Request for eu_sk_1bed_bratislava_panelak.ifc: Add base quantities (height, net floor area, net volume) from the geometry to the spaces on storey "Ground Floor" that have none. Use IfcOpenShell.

First a look at what the model holds.

```python
import ifcopenshell
import ifcopenshell.util.element
import ifcopenshell.util.unit

model = ifcopenshell.open("eu_sk_1bed_bratislava_panelak.ifc")
print(model.schema)
for unit_type in ("LENGTHUNIT", "AREAUNIT", "VOLUMEUNIT"):
    print(unit_type, ifcopenshell.util.unit.calculate_unit_scale(model, unit_type))
storey = next(s for s in model.by_type("IfcBuildingStorey") if s.Name == "Ground Floor")
spaces = [e for e in ifcopenshell.util.element.get_decomposition(storey) if e.is_a("IfcSpace")]
for e in sorted(spaces, key=lambda e: e.id()):
    print(e.id(), e.is_a(), e.Name, list(ifcopenshell.util.element.get_psets(e, qtos_only=True)), sep=" | ")
```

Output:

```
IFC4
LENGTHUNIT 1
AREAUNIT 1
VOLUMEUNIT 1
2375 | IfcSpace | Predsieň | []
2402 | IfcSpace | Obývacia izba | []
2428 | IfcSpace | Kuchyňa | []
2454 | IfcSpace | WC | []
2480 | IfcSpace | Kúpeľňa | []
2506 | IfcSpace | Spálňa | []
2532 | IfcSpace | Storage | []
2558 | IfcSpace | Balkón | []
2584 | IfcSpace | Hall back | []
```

```python
import ifcopenshell
import ifcopenshell.api.pset
import ifcopenshell.geom
import ifcopenshell.util.element
import ifcopenshell.util.shape
import ifcopenshell.util.unit

model = ifcopenshell.open("eu_sk_1bed_bratislava_panelak.ifc")
unit_scale = ifcopenshell.util.unit.calculate_unit_scale(model)
area_scale = ifcopenshell.util.unit.calculate_unit_scale(model, "AREAUNIT")
volume_scale = ifcopenshell.util.unit.calculate_unit_scale(model, "VOLUMEUNIT")
settings = ifcopenshell.geom.settings()

storey = next(s for s in model.by_type("IfcBuildingStorey") if s.Name == "Ground Floor")
spaces = [e for e in ifcopenshell.util.element.get_decomposition(storey) if e.is_a("IfcSpace")]

for e in sorted(spaces, key=lambda e: e.id()):
    if ifcopenshell.util.element.get_psets(e, qtos_only=True, should_inherit=False):
        continue
    # Geometry comes back in metres, in the element's own axes.
    shape = ifcopenshell.geom.create_shape(settings, e)
    values = {
        "Height": ifcopenshell.util.shape.get_z(shape.geometry) / unit_scale,
        "NetFloorArea": ifcopenshell.util.shape.get_footprint_area(shape.geometry) / area_scale,
        "NetVolume": ifcopenshell.util.shape.get_volume(shape.geometry) / volume_scale,
    }
    qto = ifcopenshell.api.pset.add_qto(model, product=e, name="Qto_SpaceBaseQuantities")
    ifcopenshell.api.pset.edit_qto(model, qto=qto, properties=values)
    print(e.id(), {k: round(v, 3) for k, v in values.items()})

model.write("eu_sk_1bed_bratislava_panelak_rev.ifc")
```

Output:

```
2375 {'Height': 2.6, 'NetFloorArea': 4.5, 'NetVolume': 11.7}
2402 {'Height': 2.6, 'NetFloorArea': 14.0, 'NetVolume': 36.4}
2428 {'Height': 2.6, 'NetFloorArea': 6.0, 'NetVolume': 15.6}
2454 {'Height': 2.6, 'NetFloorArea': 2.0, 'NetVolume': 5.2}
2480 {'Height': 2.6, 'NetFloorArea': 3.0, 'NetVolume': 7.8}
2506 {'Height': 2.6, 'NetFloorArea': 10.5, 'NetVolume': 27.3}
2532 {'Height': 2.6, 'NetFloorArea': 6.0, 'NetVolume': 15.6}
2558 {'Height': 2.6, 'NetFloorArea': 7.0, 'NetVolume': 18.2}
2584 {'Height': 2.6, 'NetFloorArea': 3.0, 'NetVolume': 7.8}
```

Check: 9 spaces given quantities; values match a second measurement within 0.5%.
